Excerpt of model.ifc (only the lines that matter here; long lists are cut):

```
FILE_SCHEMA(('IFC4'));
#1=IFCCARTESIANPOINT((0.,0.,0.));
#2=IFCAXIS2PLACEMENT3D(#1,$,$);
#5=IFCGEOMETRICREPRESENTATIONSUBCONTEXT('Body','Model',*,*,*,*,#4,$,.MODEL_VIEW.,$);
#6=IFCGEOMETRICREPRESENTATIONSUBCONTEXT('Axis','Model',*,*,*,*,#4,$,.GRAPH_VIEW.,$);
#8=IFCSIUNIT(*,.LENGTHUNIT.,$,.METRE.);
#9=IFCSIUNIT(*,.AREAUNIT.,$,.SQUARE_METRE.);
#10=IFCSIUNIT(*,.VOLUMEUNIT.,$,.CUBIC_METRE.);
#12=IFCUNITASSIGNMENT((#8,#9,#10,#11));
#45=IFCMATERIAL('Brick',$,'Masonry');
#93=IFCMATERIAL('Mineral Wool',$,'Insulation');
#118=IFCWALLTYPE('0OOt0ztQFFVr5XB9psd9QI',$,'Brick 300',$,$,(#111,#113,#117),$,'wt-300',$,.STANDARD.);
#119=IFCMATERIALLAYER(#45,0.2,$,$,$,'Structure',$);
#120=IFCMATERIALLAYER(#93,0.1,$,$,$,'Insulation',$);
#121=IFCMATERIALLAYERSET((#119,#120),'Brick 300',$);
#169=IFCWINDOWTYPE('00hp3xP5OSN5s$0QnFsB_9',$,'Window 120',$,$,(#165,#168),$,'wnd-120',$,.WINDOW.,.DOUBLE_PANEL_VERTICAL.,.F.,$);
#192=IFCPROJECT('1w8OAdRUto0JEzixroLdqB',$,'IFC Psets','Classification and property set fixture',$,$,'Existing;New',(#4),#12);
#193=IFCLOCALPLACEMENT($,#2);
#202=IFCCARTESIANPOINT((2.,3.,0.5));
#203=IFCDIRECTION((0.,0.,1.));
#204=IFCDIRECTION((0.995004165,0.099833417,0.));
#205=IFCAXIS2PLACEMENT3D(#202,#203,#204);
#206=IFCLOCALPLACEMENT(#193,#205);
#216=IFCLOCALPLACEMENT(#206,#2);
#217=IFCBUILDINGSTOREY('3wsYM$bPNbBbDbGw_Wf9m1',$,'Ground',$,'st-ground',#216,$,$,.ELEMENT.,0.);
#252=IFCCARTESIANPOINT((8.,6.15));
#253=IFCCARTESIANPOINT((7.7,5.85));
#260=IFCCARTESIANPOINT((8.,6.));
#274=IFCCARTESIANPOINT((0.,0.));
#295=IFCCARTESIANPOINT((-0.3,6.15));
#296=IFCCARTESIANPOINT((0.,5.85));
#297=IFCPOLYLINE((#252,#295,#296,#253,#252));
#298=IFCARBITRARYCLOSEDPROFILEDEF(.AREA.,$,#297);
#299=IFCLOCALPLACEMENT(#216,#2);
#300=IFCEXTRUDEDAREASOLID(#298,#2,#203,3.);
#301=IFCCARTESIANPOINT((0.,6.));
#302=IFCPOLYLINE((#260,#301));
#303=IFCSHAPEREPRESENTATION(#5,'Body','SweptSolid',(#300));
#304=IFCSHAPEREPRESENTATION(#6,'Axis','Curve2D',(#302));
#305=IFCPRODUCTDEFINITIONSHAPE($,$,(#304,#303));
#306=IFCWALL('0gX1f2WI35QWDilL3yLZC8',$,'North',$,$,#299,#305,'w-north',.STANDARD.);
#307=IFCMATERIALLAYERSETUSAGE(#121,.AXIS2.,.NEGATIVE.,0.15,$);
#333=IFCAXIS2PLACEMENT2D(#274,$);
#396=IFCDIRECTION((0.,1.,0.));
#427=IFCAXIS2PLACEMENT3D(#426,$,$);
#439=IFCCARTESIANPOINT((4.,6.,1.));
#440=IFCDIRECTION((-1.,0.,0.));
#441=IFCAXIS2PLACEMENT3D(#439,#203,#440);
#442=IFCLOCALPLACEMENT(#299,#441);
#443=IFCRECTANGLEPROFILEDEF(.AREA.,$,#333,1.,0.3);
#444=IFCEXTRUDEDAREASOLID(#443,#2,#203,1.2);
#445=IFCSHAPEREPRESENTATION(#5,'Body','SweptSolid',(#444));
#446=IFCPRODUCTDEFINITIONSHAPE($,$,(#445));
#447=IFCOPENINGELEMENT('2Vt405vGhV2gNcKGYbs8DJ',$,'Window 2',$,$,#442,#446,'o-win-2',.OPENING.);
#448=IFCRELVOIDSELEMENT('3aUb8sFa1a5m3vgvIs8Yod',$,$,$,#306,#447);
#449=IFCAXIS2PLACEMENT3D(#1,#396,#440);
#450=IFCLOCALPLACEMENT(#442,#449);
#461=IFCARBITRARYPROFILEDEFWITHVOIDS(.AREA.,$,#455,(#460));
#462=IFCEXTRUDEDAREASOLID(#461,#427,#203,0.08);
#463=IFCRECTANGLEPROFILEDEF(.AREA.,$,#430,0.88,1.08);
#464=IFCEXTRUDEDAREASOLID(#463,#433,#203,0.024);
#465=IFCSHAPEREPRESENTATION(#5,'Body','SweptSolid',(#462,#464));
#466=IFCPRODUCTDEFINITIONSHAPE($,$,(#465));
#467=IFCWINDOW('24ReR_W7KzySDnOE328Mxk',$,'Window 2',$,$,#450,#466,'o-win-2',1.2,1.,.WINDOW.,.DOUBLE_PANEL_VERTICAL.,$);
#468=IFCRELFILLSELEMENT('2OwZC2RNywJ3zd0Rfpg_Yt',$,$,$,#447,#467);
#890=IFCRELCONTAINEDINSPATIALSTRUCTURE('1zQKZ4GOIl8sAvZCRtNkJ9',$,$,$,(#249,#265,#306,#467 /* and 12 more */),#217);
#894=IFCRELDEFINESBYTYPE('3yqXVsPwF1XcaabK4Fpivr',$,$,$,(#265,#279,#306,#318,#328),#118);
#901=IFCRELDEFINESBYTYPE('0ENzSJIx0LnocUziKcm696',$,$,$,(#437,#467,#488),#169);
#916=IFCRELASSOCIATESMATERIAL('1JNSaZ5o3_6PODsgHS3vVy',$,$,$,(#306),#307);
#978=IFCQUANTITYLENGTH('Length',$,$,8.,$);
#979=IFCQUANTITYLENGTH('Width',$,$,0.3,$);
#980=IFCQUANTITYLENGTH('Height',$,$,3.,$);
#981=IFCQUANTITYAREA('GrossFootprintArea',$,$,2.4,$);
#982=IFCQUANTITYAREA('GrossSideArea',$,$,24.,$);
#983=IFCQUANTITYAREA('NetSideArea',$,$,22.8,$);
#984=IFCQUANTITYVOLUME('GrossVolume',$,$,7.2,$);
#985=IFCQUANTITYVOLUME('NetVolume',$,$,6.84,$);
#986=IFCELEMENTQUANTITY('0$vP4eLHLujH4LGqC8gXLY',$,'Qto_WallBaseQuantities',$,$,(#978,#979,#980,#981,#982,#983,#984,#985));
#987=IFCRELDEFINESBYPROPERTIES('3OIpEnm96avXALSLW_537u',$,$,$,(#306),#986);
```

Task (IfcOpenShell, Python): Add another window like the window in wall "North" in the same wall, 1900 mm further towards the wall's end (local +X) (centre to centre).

```python
import ifcopenshell
import ifcopenshell.api.feature
import ifcopenshell.api.geometry
import ifcopenshell.api.pset
import ifcopenshell.api.root
import ifcopenshell.geom
import ifcopenshell.util.element
import ifcopenshell.util.placement
import ifcopenshell.util.shape
import ifcopenshell.util.unit

model = ifcopenshell.open("model.ifc")
unit_scale = ifcopenshell.util.unit.calculate_unit_scale(model)
area_scale = ifcopenshell.util.unit.calculate_unit_scale(model, "AREAUNIT")
volume_scale = ifcopenshell.util.unit.calculate_unit_scale(model, "VOLUMEUNIT")
settings = ifcopenshell.geom.settings()


def volume(element):
    """Net volume in cubic metres, openings subtracted."""
    shape = ifcopenshell.geom.create_shape(settings, element)
    return ifcopenshell.util.shape.get_volume(shape.geometry)


window = model.by_guid("24ReR_W7KzySDnOE328Mxk")
opening = window.FillsVoids[0].RelatingOpeningElement
wall = opening.VoidsElements[0].RelatingBuildingElement
before = volume(wall)
shift = ifcopenshell.util.placement.get_local_placement(wall.ObjectPlacement)[:3, 0] * 1.9 / unit_scale

# copy_class copies the void relationship, type, container and properties, but no geometry.
new_opening = ifcopenshell.api.root.copy_class(model, product=opening)
new_opening.Representation = ifcopenshell.util.element.copy_deep(
    model, opening.Representation, exclude=["IfcGeometricRepresentationContext", "IfcRepresentationMap"]
)
new_opening.Tag = None
new_window = ifcopenshell.api.root.copy_class(model, product=window)
new_window.Representation = ifcopenshell.util.element.copy_deep(
    model, window.Representation, exclude=["IfcGeometricRepresentationContext", "IfcRepresentationMap"]
)
new_window.Tag = None
ifcopenshell.api.feature.add_filling(model, opening=new_opening, element=new_window)

for old, new in ((opening, new_opening), (window, new_window)):
    matrix = ifcopenshell.util.placement.get_local_placement(old.ObjectPlacement)
    matrix[:3, 3] += shift
    ifcopenshell.api.geometry.edit_object_placement(model, product=new, matrix=matrix, is_si=False)

after = volume(wall)
thickness = 0.3  # wall thickness in metres

# Update the wall's stored quantities.
qto = model.by_id(ifcopenshell.util.element.get_pset(wall, "Qto_WallBaseQuantities", should_inherit=False)["id"])
ifcopenshell.api.pset.edit_qto(model, qto=qto, properties={
    "NetSideArea": after / thickness / area_scale,
    "NetVolume": after / volume_scale,
})

print(f"wall volume {before:.3f} -> {after:.3f} m3")

model.write("model_rev.ifc")
```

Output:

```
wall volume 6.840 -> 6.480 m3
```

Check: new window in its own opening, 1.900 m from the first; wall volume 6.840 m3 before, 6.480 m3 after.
